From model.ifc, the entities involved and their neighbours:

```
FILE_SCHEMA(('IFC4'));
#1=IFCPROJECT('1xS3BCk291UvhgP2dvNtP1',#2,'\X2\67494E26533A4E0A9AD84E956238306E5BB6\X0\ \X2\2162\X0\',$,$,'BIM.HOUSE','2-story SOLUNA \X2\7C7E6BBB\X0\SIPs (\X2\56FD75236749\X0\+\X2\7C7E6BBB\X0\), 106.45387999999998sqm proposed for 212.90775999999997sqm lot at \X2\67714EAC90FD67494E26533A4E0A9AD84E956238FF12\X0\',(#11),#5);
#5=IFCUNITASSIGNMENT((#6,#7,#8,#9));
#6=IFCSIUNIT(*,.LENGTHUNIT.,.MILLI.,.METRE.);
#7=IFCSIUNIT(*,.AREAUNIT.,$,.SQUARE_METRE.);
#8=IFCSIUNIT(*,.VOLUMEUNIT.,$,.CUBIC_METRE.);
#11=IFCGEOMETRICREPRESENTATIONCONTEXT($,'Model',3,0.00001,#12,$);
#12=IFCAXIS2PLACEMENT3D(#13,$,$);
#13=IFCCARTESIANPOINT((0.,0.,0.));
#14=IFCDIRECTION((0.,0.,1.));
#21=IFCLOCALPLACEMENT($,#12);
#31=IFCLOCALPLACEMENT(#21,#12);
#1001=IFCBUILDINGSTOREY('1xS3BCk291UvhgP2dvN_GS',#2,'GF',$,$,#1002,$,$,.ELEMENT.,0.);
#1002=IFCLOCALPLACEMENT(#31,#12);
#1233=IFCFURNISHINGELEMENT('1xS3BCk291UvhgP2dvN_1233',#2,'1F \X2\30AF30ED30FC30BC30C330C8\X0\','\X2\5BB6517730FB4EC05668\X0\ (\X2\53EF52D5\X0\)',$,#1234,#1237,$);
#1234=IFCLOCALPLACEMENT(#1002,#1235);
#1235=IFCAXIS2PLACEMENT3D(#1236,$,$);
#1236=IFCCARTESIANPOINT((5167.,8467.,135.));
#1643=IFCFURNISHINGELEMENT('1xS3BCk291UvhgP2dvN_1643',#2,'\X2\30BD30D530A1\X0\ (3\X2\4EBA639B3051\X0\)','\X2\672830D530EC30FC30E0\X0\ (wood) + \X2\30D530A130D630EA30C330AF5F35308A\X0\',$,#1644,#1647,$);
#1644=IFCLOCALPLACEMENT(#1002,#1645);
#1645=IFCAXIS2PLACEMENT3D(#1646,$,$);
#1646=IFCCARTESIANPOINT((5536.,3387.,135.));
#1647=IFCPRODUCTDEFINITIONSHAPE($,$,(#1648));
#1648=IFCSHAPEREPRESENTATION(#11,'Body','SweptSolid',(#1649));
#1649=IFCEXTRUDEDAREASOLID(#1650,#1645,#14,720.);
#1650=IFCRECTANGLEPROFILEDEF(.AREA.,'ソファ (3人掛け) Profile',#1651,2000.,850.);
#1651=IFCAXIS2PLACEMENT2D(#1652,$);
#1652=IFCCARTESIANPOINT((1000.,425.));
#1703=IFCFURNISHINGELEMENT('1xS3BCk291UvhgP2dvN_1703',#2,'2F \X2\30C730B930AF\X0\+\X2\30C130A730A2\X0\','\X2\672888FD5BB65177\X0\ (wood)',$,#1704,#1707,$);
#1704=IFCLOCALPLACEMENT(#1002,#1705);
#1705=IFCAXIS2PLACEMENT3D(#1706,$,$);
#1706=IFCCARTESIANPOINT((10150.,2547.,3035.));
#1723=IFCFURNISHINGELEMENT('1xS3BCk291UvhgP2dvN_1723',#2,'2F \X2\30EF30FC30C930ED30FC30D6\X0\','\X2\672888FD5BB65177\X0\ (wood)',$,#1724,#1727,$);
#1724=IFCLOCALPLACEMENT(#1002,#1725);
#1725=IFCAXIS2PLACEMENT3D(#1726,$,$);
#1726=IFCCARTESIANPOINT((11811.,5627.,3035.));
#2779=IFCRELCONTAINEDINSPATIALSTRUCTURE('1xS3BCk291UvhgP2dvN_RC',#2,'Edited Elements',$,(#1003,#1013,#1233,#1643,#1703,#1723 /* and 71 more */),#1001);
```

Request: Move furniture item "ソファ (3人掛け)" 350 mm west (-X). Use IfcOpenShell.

```python
import ifcopenshell
import ifcopenshell.api.geometry
import ifcopenshell.util.placement
import ifcopenshell.util.unit

model = ifcopenshell.open("model.ifc")
unit_scale = ifcopenshell.util.unit.calculate_unit_scale(model)

item = model.by_guid("1xS3BCk291UvhgP2dvN_1643")
matrix = ifcopenshell.util.placement.get_local_placement(item.ObjectPlacement)
matrix[0, 3] -= 0.35 / unit_scale
ifcopenshell.api.geometry.edit_object_placement(model, product=item, matrix=matrix, is_si=False)

print(ifcopenshell.util.placement.get_local_placement(item.ObjectPlacement).round(3) + 0.0)

model.write("model_rev.ifc")
```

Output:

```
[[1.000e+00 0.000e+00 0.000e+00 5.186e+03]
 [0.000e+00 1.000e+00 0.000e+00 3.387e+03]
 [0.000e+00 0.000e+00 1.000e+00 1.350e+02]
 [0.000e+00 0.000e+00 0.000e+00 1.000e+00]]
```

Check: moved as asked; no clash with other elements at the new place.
